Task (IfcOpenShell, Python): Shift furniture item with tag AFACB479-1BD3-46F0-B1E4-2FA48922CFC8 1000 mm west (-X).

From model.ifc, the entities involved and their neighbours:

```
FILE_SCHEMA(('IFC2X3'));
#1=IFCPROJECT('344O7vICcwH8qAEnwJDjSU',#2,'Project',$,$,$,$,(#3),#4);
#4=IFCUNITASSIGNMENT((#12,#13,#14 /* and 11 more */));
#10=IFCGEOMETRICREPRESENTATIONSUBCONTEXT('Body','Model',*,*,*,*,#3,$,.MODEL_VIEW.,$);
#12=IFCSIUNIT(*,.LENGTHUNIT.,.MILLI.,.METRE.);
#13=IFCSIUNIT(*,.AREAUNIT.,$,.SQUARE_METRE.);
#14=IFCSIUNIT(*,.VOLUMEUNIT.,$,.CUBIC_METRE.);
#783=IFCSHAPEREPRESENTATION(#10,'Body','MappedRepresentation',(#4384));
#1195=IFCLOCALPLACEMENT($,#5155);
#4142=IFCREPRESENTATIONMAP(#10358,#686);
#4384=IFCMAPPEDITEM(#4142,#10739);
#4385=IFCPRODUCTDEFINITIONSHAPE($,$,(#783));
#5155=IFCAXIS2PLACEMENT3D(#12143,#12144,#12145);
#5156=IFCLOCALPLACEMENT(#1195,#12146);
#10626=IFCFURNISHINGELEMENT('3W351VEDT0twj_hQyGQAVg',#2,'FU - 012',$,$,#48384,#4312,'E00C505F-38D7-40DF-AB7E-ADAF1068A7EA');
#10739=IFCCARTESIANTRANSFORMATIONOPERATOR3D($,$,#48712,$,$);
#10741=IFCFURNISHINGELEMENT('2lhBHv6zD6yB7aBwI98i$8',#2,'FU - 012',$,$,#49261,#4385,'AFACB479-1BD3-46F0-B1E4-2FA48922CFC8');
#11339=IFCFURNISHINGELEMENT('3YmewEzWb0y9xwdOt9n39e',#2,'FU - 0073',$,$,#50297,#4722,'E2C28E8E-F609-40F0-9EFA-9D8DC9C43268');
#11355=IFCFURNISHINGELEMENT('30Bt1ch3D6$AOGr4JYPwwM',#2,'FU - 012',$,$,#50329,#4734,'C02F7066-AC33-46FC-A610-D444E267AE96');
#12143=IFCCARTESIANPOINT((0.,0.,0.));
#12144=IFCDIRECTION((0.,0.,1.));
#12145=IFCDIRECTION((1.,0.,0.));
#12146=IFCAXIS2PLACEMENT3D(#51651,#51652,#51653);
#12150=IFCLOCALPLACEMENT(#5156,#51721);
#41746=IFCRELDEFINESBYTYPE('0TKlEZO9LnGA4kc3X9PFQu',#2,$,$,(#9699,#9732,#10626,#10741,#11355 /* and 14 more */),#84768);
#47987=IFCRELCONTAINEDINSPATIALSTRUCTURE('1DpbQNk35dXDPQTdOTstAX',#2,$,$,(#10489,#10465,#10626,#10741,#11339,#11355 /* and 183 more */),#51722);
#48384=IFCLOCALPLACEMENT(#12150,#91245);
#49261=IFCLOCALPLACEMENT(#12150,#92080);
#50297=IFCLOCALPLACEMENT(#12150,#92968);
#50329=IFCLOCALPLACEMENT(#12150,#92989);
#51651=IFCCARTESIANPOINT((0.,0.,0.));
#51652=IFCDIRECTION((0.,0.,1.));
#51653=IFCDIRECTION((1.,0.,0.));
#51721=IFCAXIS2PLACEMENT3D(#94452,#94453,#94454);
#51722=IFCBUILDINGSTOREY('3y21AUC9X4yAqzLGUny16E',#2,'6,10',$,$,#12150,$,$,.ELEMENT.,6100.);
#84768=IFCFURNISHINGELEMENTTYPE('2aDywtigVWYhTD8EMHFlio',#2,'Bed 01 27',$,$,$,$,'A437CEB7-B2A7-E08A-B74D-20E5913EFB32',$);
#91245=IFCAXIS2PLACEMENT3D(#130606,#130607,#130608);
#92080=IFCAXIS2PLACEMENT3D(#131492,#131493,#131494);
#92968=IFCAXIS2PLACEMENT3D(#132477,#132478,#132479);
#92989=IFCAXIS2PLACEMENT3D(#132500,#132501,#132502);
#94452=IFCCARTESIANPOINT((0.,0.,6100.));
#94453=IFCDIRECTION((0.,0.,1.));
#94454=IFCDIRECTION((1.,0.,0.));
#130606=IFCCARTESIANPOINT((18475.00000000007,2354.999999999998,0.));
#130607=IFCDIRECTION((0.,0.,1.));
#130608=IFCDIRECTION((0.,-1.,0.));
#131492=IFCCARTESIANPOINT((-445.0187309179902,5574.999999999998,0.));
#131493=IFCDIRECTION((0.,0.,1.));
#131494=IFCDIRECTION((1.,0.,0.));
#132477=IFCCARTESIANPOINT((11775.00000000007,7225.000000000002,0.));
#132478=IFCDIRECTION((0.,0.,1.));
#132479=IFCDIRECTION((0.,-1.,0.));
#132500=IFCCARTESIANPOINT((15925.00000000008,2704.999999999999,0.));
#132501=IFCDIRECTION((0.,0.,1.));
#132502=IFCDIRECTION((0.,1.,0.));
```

```python
import ifcopenshell
import ifcopenshell.api.geometry
import ifcopenshell.util.placement

model = ifcopenshell.open("model.ifc")

item = model.by_guid("2lhBHv6zD6yB7aBwI98i$8")
matrix = ifcopenshell.util.placement.get_local_placement(item.ObjectPlacement)
matrix[0, 3] -= 1000.0
ifcopenshell.api.geometry.edit_object_placement(model, product=item, matrix=matrix, is_si=False)

print(ifcopenshell.util.placement.get_local_placement(item.ObjectPlacement).round(3) + 0.0)

model.write("model_updated.ifc")
```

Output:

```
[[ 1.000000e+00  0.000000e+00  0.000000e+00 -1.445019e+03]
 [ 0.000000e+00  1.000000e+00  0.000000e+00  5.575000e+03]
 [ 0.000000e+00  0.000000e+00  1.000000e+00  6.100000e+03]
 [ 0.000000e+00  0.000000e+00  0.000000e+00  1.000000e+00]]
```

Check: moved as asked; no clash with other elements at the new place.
